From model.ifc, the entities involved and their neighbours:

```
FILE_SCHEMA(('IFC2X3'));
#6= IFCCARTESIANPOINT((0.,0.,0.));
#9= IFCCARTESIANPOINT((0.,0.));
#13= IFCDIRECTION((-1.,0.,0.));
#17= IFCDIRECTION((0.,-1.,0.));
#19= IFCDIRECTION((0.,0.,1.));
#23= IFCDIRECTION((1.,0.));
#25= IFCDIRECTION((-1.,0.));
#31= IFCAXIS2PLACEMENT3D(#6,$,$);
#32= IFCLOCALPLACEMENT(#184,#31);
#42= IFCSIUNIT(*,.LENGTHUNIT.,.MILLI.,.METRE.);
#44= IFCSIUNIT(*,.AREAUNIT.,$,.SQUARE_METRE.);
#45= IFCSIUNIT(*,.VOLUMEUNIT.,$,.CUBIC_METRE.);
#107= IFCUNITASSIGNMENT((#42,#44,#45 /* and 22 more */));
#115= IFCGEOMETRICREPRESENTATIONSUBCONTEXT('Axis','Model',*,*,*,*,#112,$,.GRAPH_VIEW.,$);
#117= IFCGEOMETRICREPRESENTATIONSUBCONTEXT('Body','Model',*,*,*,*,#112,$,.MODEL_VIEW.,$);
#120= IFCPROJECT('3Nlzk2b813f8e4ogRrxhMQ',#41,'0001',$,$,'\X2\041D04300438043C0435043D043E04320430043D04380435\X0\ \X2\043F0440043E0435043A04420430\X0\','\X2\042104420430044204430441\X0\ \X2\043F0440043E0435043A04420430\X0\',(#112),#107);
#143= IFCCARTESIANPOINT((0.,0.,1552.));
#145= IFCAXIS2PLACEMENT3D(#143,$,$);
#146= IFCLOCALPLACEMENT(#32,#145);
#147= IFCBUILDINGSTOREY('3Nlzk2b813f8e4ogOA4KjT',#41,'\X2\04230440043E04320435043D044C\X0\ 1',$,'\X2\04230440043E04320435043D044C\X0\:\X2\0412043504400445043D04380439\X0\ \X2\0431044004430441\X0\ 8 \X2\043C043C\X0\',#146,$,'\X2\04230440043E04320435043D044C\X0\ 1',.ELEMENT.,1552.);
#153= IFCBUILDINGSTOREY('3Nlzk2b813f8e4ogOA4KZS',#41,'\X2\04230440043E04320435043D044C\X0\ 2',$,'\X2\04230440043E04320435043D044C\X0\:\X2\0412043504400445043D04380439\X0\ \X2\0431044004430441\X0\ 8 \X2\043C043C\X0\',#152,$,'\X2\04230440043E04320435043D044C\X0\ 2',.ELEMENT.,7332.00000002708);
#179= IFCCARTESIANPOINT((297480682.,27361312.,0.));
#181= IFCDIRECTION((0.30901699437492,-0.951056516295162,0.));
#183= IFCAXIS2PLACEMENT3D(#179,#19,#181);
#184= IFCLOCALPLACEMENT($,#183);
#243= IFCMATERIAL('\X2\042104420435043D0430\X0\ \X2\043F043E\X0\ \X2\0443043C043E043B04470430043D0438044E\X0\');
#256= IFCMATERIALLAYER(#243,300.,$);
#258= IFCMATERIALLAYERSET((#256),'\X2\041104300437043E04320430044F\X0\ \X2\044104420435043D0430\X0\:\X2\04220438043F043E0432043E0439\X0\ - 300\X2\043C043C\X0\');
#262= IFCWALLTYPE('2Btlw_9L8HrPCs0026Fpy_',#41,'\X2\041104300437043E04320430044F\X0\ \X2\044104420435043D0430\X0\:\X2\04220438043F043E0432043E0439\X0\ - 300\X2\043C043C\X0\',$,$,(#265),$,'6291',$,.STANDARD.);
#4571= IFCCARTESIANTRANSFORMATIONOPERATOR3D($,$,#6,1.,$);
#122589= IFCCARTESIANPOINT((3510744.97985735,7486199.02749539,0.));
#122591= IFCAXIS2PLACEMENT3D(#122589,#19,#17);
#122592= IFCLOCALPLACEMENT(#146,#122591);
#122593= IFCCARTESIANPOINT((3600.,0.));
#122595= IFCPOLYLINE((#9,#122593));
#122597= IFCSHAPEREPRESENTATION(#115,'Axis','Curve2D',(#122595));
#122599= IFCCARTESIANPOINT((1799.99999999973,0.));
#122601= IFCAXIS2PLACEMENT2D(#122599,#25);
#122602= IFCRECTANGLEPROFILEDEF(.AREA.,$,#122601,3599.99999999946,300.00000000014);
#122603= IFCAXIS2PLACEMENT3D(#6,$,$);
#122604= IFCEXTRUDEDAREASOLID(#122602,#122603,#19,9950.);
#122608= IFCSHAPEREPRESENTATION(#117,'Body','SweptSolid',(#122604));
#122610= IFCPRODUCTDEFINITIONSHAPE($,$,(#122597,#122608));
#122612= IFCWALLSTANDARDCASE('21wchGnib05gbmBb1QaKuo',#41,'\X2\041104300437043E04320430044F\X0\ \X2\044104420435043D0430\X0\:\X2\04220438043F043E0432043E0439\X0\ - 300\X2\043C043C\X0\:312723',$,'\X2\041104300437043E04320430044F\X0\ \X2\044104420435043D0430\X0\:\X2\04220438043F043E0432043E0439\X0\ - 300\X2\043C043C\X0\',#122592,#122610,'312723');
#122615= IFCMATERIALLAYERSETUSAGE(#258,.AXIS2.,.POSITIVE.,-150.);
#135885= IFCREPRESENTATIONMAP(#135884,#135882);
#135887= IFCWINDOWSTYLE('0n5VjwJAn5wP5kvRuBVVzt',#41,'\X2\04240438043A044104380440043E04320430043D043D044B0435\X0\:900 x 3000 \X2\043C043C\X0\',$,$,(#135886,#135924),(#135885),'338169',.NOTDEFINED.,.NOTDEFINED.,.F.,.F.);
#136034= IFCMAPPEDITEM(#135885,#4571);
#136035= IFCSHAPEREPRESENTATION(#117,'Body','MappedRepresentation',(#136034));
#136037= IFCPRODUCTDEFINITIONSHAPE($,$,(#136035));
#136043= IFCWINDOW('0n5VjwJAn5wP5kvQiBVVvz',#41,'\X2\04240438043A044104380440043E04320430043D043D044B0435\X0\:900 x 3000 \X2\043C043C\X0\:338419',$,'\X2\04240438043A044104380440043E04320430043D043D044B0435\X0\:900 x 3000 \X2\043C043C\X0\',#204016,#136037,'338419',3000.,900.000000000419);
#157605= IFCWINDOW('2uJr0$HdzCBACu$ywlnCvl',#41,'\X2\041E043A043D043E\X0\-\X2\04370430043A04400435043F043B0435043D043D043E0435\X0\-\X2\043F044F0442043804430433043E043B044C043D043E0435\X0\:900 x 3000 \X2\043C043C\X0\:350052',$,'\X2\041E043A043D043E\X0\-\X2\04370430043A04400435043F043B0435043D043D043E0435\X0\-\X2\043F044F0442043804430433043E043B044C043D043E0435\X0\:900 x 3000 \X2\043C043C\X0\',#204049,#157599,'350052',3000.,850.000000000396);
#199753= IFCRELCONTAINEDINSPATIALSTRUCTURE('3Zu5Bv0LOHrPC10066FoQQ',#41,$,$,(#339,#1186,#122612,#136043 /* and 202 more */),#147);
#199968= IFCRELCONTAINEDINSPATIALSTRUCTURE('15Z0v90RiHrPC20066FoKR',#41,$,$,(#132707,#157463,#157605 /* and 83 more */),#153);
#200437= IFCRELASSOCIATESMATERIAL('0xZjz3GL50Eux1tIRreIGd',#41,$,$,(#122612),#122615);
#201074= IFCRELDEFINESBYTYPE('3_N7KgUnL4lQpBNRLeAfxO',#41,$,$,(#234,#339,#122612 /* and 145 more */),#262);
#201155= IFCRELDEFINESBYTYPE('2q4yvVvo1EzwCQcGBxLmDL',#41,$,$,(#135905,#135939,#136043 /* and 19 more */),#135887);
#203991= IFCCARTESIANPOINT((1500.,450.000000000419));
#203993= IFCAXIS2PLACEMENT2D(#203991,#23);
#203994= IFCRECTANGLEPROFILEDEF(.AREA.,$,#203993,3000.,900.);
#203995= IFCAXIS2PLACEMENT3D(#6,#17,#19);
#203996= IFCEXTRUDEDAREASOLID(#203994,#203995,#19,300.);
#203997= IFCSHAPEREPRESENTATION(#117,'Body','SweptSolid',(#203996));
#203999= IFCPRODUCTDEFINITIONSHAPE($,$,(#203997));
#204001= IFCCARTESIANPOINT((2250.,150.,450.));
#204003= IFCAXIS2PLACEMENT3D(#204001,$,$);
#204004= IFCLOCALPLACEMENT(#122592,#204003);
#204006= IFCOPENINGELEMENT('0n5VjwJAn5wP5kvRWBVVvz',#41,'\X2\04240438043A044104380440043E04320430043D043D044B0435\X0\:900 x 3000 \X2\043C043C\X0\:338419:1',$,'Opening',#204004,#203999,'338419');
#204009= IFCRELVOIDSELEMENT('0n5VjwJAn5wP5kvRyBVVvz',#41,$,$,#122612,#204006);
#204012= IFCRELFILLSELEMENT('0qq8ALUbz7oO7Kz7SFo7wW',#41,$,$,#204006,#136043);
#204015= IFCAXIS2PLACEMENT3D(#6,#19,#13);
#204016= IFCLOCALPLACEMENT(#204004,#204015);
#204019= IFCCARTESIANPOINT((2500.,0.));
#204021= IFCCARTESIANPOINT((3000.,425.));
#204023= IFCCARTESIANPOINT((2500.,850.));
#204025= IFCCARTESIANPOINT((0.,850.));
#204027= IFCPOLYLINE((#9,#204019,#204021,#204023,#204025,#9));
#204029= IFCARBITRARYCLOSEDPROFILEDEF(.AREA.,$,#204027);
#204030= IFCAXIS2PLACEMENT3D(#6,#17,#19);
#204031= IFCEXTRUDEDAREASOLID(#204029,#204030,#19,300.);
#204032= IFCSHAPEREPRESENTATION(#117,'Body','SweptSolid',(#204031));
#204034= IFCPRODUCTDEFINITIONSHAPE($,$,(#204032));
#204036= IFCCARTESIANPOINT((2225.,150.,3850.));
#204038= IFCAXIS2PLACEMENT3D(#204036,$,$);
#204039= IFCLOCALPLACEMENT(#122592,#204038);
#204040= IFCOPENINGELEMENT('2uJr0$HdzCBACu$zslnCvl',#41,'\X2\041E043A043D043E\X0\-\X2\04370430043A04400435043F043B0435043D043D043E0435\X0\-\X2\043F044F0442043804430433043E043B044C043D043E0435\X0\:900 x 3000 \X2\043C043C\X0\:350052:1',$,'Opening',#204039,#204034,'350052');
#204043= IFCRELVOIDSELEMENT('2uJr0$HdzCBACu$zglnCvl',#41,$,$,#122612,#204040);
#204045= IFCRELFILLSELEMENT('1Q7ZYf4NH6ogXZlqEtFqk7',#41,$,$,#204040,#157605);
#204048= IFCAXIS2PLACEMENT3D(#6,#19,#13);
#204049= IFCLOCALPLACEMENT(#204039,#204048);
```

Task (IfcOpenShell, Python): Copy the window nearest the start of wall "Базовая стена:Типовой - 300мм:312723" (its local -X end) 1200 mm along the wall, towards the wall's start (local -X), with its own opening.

```python
import ifcopenshell
import ifcopenshell.api.feature
import ifcopenshell.api.geometry
import ifcopenshell.api.root
import ifcopenshell.geom
import ifcopenshell.util.element
import ifcopenshell.util.placement
import ifcopenshell.util.shape
import ifcopenshell.util.unit

model = ifcopenshell.open("model.ifc")
unit_scale = ifcopenshell.util.unit.calculate_unit_scale(model)
settings = ifcopenshell.geom.settings()


def volume(element):
    """Net volume in cubic metres, openings subtracted."""
    shape = ifcopenshell.geom.create_shape(settings, element)
    return ifcopenshell.util.shape.get_volume(shape.geometry)


def reuse_history(source, copy):
    """copy_class also copies each property set's owner history, people and application; keep the originals."""
    for rel in copy.IsDefinedBy:
        if rel.is_a("IfcRelDefinesByProperties") and (history := rel.RelatingPropertyDefinition.OwnerHistory):
            rel.RelatingPropertyDefinition.OwnerHistory = source.OwnerHistory
            ifcopenshell.util.element.remove_deep2(model, history)


window = model.by_id(136043)
opening = window.FillsVoids[0].RelatingOpeningElement
wall = opening.VoidsElements[0].RelatingBuildingElement
before = volume(wall)
shift = ifcopenshell.util.placement.get_local_placement(wall.ObjectPlacement)[:3, 0] * -1.2 / unit_scale

# copy_class copies the void relationship, type, container and properties, but no geometry.
new_opening = ifcopenshell.api.root.copy_class(model, product=opening)
new_opening.Representation = ifcopenshell.util.element.copy_deep(
    model, opening.Representation, exclude=["IfcGeometricRepresentationContext", "IfcRepresentationMap"]
)
new_opening.Name = "Фиксированные:900 x 3000 мм"
new_opening.Tag = None
new_window = ifcopenshell.api.root.copy_class(model, product=window)
new_window.Representation = ifcopenshell.util.element.copy_deep(
    model, window.Representation, exclude=["IfcGeometricRepresentationContext", "IfcRepresentationMap"]
)
new_window.Name = "Фиксированные:900 x 3000 мм"
new_window.Tag = None
reuse_history(window, new_window)
fills = ifcopenshell.api.feature.add_filling(model, opening=new_opening, element=new_window)
fills.OwnerHistory = new_window.OwnerHistory  # required in IFC2X3

for old, new in ((opening, new_opening), (window, new_window)):
    matrix = ifcopenshell.util.placement.get_local_placement(old.ObjectPlacement)
    matrix[:3, 3] += shift
    ifcopenshell.api.geometry.edit_object_placement(model, product=new, matrix=matrix, is_si=False)

after = volume(wall)

print(f"wall volume {before:.3f} -> {after:.3f} m3")

model.write("model-out.ifc")
```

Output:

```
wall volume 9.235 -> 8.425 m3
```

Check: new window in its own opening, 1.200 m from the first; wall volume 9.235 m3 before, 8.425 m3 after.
